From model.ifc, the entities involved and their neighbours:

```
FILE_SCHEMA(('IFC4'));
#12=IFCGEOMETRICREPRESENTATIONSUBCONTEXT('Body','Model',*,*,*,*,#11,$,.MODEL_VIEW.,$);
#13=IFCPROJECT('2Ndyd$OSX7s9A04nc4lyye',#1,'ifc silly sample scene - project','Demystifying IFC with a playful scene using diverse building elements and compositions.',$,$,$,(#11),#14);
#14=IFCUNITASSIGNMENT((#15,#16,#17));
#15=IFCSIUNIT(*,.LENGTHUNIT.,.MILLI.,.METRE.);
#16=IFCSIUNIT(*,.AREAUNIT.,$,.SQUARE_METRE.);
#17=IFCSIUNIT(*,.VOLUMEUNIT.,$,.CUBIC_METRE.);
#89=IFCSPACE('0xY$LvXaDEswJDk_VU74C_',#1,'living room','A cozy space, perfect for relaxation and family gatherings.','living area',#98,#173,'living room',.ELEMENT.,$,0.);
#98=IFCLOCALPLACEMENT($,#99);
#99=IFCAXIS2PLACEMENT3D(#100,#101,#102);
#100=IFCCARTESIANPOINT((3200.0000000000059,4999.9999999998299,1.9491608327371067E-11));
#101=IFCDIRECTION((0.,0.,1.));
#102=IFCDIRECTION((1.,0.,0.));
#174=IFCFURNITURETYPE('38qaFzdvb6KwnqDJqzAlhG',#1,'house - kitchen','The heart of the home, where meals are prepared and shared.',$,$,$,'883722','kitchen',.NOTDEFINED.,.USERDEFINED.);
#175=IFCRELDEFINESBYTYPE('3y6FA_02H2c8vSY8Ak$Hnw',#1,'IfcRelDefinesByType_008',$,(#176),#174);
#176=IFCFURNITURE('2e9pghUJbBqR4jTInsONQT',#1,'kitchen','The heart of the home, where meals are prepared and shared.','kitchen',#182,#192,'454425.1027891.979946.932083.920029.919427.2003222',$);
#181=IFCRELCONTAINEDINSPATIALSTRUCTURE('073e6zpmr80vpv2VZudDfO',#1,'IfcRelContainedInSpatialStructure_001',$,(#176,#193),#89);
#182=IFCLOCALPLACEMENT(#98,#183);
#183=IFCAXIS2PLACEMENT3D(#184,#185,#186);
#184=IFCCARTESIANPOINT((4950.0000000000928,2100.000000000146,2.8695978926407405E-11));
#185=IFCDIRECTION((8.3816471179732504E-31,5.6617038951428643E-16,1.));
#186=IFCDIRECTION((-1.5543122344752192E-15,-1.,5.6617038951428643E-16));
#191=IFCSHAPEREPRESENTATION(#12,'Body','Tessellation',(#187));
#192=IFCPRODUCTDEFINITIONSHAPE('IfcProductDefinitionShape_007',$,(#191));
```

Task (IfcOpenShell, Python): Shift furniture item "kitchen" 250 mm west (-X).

```python
import ifcopenshell
import ifcopenshell.api.geometry
import ifcopenshell.util.placement

model = ifcopenshell.open("model.ifc")

item = model.by_id(176)
matrix = ifcopenshell.util.placement.get_local_placement(item.ObjectPlacement)
matrix[0, 3] -= 250.0
ifcopenshell.api.geometry.edit_object_placement(model, product=item, matrix=matrix, is_si=False)

print(ifcopenshell.util.placement.get_local_placement(item.ObjectPlacement).round(3) + 0.0)

model.write("model_edited.ifc")
```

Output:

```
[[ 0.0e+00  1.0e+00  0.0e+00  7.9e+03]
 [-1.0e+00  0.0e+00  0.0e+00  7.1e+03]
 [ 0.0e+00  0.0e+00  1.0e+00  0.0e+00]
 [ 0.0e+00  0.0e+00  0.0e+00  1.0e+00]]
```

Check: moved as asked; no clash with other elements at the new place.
